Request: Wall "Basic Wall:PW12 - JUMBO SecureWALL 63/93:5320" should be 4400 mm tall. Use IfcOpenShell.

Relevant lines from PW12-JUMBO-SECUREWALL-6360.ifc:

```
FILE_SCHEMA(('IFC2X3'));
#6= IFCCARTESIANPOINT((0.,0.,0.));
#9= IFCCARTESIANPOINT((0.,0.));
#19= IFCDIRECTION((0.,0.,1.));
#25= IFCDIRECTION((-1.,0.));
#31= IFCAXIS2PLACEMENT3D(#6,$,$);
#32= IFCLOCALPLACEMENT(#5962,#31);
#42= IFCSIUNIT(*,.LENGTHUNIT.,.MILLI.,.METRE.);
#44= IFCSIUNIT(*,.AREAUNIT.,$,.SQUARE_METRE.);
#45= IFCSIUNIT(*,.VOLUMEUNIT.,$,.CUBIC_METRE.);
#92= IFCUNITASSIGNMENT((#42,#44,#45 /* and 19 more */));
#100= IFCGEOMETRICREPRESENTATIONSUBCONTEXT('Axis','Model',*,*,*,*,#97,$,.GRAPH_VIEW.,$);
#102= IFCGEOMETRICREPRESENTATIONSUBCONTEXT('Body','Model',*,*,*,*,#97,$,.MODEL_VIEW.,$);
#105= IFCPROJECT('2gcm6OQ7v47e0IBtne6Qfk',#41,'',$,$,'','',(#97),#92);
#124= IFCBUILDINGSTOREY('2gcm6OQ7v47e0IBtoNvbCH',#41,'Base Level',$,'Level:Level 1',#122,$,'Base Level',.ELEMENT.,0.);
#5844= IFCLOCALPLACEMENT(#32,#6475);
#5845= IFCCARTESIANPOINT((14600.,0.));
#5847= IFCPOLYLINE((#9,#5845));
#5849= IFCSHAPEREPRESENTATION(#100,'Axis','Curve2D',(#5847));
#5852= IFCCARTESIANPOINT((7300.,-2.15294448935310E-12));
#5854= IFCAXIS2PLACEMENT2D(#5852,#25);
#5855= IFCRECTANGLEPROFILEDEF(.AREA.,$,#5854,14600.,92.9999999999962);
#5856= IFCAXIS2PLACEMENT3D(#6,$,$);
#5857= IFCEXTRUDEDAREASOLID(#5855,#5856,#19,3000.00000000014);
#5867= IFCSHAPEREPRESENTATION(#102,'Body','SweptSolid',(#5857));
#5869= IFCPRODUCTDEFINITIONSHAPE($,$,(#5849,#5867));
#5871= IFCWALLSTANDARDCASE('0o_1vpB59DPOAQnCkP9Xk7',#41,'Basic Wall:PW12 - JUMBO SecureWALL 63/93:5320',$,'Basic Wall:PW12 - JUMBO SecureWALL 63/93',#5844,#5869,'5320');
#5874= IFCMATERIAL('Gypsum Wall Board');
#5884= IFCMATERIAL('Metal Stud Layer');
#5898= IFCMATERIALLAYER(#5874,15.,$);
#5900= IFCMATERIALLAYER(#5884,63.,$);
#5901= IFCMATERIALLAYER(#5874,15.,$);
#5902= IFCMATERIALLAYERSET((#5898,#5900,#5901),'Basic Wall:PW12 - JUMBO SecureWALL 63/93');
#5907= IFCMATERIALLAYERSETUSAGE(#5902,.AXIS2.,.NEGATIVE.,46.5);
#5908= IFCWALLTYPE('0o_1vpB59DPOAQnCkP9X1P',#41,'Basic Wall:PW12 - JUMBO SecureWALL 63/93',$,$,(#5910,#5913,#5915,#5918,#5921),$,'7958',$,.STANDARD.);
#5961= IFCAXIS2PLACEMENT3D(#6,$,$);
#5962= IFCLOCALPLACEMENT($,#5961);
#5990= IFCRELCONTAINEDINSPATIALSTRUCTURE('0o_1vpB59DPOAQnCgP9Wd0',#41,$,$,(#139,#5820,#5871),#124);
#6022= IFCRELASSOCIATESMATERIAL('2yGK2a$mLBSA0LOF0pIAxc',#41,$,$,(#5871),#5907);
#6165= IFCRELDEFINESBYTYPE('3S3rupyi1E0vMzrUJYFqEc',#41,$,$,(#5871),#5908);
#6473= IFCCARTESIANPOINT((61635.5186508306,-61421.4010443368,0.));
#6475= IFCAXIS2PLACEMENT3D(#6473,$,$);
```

```python
import ifcopenshell
import ifcopenshell.geom
import ifcopenshell.util.representation
import ifcopenshell.util.shape

model = ifcopenshell.open("PW12-JUMBO-SECUREWALL-6360.ifc")
settings = ifcopenshell.geom.settings()


def volume(element):
    """Net volume in cubic metres, openings subtracted."""
    shape = ifcopenshell.geom.create_shape(settings, element)
    return ifcopenshell.util.shape.get_volume(shape.geometry)


wall = model.by_id(5871)
before = volume(wall)

body = ifcopenshell.util.representation.get_representation(wall, "Model", "Body")
solid = body.Items[0]
old_height = solid.Depth
solid.Depth = 4400.0
after = volume(wall)

print(f"height {old_height:g} -> {solid.Depth:g}, volume {before:.3f} -> {after:.3f} m3")

model.write("PW12-JUMBO-SECUREWALL-6360_rev.ifc")
```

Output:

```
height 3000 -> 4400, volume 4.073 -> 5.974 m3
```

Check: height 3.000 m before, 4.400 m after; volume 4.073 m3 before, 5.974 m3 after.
